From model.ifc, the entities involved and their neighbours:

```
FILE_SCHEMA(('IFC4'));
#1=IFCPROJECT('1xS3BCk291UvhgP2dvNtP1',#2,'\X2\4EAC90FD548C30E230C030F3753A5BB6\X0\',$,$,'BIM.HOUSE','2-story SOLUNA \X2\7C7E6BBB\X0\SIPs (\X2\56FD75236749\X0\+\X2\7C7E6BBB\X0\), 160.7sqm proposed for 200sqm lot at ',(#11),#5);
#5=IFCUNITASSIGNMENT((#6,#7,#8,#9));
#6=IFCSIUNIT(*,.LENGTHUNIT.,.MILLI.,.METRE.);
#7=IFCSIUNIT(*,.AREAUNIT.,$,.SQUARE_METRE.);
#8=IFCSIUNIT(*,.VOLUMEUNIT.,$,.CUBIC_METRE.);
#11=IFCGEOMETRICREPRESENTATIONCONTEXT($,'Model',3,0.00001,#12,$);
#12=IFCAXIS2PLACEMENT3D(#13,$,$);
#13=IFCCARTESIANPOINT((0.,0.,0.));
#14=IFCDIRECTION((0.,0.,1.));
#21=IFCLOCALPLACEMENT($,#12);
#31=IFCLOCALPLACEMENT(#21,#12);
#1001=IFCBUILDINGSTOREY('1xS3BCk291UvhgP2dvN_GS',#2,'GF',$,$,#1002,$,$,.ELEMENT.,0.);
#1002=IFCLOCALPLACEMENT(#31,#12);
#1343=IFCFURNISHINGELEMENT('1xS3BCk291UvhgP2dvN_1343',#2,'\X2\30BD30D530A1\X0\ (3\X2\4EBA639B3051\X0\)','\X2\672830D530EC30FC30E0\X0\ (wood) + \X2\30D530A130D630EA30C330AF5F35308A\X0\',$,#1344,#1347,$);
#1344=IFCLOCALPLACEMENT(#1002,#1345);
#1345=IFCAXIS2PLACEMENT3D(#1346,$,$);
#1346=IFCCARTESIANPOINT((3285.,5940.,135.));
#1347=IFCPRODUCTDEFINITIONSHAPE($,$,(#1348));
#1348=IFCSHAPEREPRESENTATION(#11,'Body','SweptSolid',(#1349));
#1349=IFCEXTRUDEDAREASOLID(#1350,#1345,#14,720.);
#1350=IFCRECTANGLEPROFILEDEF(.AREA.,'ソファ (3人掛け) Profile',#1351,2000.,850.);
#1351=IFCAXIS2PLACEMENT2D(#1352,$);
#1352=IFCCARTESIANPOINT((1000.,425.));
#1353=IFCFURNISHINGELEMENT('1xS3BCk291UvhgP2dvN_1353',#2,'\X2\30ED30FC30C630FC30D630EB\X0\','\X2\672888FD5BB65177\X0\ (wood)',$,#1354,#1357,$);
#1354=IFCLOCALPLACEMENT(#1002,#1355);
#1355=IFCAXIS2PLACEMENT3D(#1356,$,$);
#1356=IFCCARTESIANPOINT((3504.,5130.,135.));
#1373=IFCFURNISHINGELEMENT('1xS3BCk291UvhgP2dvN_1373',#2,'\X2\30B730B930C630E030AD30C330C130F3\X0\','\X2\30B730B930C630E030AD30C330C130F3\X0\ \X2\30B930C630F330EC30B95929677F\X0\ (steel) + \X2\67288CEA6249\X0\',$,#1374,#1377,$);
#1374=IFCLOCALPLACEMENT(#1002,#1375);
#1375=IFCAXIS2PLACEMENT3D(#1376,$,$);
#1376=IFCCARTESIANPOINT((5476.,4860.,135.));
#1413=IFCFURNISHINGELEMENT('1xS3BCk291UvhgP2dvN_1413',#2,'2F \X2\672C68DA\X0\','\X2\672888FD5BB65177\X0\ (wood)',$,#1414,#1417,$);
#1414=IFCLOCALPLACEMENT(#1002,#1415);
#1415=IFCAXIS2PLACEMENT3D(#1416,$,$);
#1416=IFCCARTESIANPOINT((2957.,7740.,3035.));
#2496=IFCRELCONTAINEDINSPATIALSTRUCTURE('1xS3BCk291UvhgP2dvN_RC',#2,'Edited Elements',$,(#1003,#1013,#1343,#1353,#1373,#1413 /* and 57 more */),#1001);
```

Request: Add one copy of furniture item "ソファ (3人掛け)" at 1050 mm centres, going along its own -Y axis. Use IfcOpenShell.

```python
import ifcopenshell
import ifcopenshell.api.geometry
import ifcopenshell.api.root
import ifcopenshell.util.element
import ifcopenshell.util.placement
import ifcopenshell.util.unit

model = ifcopenshell.open("model.ifc")
unit_scale = ifcopenshell.util.unit.calculate_unit_scale(model)


def reuse_history(source, copy):
    """copy_class also copies each property set's owner history, people and application; keep the originals."""
    for rel in copy.IsDefinedBy:
        if rel.is_a("IfcRelDefinesByProperties") and (history := rel.RelatingPropertyDefinition.OwnerHistory):
            rel.RelatingPropertyDefinition.OwnerHistory = source.OwnerHistory
            ifcopenshell.util.element.remove_deep2(model, history)


source = model.by_guid("1xS3BCk291UvhgP2dvN_1343")
base = ifcopenshell.util.placement.get_local_placement(source.ObjectPlacement)
step = -base[:3, 1] * 1.05 / unit_scale

for i in range(1, 2):
    copy = ifcopenshell.api.root.copy_class(model, product=source)
    copy.Representation = ifcopenshell.util.element.copy_deep(
        model, source.Representation, exclude=["IfcGeometricRepresentationContext", "IfcRepresentationMap"]
    )
    reuse_history(source, copy)
    matrix = base.copy()
    matrix[:3, 3] += i * step
    print("added at", matrix[:3, 3].round(3) + 0.0)
    ifcopenshell.api.geometry.edit_object_placement(model, product=copy, matrix=matrix, is_si=False)

model.write("model_updated.ifc")
```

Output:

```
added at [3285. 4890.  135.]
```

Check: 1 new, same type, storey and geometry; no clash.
